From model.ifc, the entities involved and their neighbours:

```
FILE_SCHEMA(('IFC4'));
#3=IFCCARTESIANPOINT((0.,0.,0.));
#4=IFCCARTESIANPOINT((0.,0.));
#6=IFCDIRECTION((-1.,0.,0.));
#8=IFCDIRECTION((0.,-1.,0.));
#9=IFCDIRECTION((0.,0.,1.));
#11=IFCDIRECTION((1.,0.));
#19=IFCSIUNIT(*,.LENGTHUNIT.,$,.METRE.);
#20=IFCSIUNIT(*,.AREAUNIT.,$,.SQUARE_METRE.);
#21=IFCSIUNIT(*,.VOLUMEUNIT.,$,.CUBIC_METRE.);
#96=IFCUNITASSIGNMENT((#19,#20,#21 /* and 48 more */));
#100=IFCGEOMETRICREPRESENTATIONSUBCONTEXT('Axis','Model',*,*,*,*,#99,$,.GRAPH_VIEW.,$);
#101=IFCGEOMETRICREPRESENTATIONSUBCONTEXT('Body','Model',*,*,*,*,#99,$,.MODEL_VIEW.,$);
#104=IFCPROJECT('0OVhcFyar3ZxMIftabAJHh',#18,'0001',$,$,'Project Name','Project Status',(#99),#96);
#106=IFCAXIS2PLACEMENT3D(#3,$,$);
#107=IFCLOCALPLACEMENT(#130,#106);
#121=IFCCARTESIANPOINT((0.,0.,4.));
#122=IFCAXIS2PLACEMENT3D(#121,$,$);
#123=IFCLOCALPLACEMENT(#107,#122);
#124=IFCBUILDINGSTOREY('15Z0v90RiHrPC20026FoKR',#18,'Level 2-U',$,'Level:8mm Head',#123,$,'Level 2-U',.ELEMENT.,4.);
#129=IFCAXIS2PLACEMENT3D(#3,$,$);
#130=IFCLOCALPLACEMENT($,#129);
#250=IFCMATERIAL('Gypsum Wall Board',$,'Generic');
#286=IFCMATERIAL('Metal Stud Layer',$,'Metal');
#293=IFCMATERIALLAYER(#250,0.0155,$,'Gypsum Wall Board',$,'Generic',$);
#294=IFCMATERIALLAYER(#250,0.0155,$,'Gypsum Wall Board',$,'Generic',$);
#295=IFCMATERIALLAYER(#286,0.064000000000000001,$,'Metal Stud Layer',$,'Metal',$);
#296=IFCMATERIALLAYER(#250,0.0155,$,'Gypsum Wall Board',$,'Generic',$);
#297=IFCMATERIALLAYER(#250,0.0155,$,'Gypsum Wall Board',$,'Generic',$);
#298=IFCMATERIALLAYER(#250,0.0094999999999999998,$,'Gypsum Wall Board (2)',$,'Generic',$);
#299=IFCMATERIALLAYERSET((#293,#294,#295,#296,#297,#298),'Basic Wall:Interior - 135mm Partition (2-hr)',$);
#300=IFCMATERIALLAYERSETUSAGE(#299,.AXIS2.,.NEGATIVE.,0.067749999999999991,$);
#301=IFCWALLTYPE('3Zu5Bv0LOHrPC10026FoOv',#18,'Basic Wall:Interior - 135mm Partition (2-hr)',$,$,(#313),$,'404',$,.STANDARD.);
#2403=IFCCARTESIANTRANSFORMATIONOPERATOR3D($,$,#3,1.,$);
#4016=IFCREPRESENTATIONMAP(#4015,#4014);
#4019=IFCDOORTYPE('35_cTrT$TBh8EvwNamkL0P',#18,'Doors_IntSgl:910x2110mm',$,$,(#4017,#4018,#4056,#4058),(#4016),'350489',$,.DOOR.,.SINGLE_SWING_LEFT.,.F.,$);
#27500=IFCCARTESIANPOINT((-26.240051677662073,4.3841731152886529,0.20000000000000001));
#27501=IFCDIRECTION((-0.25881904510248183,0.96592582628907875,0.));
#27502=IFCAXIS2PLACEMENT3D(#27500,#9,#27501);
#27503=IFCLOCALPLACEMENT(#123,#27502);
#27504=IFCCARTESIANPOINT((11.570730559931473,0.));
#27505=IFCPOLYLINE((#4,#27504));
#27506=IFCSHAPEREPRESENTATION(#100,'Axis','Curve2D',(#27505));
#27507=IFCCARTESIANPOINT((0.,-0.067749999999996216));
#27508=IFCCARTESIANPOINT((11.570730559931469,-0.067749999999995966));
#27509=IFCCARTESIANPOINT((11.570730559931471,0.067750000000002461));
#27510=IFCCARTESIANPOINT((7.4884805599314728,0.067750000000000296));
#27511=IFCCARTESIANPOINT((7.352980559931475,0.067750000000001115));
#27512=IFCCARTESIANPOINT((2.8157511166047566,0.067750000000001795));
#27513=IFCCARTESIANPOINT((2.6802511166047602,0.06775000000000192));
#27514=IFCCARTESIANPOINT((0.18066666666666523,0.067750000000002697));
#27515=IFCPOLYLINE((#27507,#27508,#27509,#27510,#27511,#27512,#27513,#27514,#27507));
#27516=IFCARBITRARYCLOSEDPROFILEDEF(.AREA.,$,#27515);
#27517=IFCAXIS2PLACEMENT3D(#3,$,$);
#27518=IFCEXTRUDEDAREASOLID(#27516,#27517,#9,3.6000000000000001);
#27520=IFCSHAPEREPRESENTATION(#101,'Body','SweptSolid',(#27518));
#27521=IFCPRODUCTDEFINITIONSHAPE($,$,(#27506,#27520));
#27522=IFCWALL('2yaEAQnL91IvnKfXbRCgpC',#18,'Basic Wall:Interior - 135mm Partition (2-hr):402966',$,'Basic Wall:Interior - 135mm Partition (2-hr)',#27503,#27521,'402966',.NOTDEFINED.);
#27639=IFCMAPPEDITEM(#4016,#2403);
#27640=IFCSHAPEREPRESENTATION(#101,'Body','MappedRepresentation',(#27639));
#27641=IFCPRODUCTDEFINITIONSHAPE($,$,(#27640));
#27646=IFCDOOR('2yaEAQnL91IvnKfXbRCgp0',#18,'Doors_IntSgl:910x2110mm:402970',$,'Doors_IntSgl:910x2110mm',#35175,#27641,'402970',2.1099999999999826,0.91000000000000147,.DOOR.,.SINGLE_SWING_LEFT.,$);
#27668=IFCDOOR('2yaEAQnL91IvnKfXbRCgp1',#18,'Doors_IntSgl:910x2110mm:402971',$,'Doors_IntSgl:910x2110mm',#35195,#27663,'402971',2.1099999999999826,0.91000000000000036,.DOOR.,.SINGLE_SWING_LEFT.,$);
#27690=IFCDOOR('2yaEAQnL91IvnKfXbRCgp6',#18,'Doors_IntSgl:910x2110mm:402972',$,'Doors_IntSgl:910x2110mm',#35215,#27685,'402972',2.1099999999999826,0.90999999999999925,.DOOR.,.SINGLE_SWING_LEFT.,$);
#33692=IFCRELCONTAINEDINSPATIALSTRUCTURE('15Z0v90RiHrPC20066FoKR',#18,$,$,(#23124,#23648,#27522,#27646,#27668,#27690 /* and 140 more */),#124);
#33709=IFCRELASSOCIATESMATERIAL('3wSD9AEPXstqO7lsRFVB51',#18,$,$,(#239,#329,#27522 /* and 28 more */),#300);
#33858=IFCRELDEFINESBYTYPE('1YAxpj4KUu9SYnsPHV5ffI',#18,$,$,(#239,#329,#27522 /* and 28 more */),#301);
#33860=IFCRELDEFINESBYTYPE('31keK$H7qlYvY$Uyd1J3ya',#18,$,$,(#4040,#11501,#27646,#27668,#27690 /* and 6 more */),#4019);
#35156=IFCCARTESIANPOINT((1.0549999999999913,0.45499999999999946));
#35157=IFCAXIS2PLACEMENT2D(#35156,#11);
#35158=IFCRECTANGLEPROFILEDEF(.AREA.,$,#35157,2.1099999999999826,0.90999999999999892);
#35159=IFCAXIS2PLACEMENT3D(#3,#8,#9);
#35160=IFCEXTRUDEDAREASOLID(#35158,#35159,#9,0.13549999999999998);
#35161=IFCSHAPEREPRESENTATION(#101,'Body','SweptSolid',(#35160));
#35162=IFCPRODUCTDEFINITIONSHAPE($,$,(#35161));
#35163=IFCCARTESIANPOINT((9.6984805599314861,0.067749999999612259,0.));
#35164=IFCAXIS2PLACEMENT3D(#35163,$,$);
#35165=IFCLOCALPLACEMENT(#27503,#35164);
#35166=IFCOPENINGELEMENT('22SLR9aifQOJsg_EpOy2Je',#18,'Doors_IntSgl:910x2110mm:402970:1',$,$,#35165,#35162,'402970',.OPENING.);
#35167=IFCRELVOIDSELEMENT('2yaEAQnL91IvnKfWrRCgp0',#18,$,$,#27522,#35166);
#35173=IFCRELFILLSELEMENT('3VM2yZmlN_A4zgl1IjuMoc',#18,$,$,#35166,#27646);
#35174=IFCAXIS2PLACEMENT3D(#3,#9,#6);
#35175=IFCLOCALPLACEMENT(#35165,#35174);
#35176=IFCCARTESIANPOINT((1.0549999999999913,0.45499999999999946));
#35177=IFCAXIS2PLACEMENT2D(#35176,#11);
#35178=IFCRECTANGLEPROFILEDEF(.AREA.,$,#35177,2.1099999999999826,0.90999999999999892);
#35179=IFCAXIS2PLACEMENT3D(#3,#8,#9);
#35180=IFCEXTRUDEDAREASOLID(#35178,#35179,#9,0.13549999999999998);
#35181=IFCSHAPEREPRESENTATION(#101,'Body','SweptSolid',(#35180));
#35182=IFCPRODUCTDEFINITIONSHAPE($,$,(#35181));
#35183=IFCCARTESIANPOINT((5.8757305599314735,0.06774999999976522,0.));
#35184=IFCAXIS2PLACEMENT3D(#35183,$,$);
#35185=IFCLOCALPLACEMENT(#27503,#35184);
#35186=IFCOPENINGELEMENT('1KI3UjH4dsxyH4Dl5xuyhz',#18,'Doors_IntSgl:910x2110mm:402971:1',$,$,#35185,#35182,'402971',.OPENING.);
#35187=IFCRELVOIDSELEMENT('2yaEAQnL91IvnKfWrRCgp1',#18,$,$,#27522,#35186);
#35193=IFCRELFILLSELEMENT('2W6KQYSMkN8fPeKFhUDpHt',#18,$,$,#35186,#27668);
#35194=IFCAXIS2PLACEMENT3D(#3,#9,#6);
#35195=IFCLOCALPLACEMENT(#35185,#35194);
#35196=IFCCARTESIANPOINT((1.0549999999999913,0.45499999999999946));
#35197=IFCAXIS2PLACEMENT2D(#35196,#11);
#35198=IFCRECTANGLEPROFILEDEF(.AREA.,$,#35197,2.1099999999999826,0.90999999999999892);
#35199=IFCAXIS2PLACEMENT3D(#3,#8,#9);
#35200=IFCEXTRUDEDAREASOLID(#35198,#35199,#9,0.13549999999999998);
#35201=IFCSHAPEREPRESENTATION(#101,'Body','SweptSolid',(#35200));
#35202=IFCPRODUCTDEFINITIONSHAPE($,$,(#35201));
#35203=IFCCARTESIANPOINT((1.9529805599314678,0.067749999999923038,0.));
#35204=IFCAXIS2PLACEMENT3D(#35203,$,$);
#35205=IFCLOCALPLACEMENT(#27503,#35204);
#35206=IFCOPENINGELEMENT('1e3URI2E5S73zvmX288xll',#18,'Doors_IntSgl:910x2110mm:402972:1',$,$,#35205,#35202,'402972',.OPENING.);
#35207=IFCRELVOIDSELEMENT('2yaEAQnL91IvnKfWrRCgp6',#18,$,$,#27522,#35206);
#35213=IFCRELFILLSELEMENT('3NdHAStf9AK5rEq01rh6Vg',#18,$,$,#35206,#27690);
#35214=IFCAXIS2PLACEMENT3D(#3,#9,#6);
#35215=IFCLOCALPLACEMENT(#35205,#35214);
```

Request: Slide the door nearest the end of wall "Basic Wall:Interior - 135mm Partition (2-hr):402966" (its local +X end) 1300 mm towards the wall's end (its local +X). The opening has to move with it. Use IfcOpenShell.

```python
import ifcopenshell
import ifcopenshell.api.geometry
import ifcopenshell.util.placement

model = ifcopenshell.open("model.ifc")

door = model.by_id(27646)
opening = door.FillsVoids[0].RelatingOpeningElement
wall = opening.VoidsElements[0].RelatingBuildingElement

wall_matrix = ifcopenshell.util.placement.get_local_placement(wall.ObjectPlacement)
shift = wall_matrix[:3, 0] * 1.3
before = ifcopenshell.util.placement.get_local_placement(door.ObjectPlacement)[:3, 3].copy()

# The door is placed relative to its opening, so it follows when the opening moves.
matrix = ifcopenshell.util.placement.get_local_placement(opening.ObjectPlacement)
matrix[:3, 3] += shift
ifcopenshell.api.geometry.edit_object_placement(
    model, product=opening, matrix=matrix, is_si=False, should_transform_children=True
)

after = ifcopenshell.util.placement.get_local_placement(door.ObjectPlacement)[:3, 3]
print("door moved by", (after - before).round(3) + 0.0)

model.write("model-out.ifc")
```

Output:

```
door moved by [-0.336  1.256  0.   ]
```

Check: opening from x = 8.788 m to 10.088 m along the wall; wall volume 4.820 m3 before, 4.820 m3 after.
